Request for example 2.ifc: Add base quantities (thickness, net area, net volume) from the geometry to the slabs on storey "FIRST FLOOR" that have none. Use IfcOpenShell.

First a look at what the model holds.

```python
import ifcopenshell
import ifcopenshell.util.element
import ifcopenshell.util.unit

model = ifcopenshell.open("example 2.ifc")
print(model.schema)
for unit_type in ("LENGTHUNIT", "AREAUNIT", "VOLUMEUNIT"):
    print(unit_type, ifcopenshell.util.unit.calculate_unit_scale(model, unit_type))
storey = next(s for s in model.by_type("IfcBuildingStorey") if s.Name == "FIRST FLOOR")
slabs = [e for e in ifcopenshell.util.element.get_decomposition(storey) if e.is_a("IfcSlab")]
for e in sorted(slabs, key=lambda e: e.id()):
    print(e.id(), e.is_a(), e.Name, list(ifcopenshell.util.element.get_psets(e, qtos_only=True)), sep=" | ")
```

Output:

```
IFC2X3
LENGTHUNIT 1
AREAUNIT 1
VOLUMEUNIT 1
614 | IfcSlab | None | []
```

```python
import ifcopenshell
import ifcopenshell.api.pset
import ifcopenshell.geom
import ifcopenshell.util.element
import ifcopenshell.util.shape
import ifcopenshell.util.unit

model = ifcopenshell.open("example 2.ifc")
unit_scale = ifcopenshell.util.unit.calculate_unit_scale(model)
area_scale = ifcopenshell.util.unit.calculate_unit_scale(model, "AREAUNIT")
volume_scale = ifcopenshell.util.unit.calculate_unit_scale(model, "VOLUMEUNIT")
settings = ifcopenshell.geom.settings()

storey = next(s for s in model.by_type("IfcBuildingStorey") if s.Name == "FIRST FLOOR")
slabs = [e for e in ifcopenshell.util.element.get_decomposition(storey) if e.is_a("IfcSlab")]

for e in sorted(slabs, key=lambda e: e.id()):
    if ifcopenshell.util.element.get_psets(e, qtos_only=True, should_inherit=False):
        continue
    # Geometry comes back in metres, in the element's own axes.
    shape = ifcopenshell.geom.create_shape(settings, e)
    values = {
        "Width": ifcopenshell.util.shape.get_z(shape.geometry) / unit_scale,
        "NetArea": ifcopenshell.util.shape.get_footprint_area(shape.geometry) / area_scale,
        "NetVolume": ifcopenshell.util.shape.get_volume(shape.geometry) / volume_scale,
    }
    qto = ifcopenshell.api.pset.add_qto(model, product=e, name="BaseQuantities")
    ifcopenshell.api.pset.edit_qto(model, qto=qto, properties=values)
    print(e.id(), {k: round(v, 3) for k, v in values.items()})

model.write("example 2-out.ifc")
```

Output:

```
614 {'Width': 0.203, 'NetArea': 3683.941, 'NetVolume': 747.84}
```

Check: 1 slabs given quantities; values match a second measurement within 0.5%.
